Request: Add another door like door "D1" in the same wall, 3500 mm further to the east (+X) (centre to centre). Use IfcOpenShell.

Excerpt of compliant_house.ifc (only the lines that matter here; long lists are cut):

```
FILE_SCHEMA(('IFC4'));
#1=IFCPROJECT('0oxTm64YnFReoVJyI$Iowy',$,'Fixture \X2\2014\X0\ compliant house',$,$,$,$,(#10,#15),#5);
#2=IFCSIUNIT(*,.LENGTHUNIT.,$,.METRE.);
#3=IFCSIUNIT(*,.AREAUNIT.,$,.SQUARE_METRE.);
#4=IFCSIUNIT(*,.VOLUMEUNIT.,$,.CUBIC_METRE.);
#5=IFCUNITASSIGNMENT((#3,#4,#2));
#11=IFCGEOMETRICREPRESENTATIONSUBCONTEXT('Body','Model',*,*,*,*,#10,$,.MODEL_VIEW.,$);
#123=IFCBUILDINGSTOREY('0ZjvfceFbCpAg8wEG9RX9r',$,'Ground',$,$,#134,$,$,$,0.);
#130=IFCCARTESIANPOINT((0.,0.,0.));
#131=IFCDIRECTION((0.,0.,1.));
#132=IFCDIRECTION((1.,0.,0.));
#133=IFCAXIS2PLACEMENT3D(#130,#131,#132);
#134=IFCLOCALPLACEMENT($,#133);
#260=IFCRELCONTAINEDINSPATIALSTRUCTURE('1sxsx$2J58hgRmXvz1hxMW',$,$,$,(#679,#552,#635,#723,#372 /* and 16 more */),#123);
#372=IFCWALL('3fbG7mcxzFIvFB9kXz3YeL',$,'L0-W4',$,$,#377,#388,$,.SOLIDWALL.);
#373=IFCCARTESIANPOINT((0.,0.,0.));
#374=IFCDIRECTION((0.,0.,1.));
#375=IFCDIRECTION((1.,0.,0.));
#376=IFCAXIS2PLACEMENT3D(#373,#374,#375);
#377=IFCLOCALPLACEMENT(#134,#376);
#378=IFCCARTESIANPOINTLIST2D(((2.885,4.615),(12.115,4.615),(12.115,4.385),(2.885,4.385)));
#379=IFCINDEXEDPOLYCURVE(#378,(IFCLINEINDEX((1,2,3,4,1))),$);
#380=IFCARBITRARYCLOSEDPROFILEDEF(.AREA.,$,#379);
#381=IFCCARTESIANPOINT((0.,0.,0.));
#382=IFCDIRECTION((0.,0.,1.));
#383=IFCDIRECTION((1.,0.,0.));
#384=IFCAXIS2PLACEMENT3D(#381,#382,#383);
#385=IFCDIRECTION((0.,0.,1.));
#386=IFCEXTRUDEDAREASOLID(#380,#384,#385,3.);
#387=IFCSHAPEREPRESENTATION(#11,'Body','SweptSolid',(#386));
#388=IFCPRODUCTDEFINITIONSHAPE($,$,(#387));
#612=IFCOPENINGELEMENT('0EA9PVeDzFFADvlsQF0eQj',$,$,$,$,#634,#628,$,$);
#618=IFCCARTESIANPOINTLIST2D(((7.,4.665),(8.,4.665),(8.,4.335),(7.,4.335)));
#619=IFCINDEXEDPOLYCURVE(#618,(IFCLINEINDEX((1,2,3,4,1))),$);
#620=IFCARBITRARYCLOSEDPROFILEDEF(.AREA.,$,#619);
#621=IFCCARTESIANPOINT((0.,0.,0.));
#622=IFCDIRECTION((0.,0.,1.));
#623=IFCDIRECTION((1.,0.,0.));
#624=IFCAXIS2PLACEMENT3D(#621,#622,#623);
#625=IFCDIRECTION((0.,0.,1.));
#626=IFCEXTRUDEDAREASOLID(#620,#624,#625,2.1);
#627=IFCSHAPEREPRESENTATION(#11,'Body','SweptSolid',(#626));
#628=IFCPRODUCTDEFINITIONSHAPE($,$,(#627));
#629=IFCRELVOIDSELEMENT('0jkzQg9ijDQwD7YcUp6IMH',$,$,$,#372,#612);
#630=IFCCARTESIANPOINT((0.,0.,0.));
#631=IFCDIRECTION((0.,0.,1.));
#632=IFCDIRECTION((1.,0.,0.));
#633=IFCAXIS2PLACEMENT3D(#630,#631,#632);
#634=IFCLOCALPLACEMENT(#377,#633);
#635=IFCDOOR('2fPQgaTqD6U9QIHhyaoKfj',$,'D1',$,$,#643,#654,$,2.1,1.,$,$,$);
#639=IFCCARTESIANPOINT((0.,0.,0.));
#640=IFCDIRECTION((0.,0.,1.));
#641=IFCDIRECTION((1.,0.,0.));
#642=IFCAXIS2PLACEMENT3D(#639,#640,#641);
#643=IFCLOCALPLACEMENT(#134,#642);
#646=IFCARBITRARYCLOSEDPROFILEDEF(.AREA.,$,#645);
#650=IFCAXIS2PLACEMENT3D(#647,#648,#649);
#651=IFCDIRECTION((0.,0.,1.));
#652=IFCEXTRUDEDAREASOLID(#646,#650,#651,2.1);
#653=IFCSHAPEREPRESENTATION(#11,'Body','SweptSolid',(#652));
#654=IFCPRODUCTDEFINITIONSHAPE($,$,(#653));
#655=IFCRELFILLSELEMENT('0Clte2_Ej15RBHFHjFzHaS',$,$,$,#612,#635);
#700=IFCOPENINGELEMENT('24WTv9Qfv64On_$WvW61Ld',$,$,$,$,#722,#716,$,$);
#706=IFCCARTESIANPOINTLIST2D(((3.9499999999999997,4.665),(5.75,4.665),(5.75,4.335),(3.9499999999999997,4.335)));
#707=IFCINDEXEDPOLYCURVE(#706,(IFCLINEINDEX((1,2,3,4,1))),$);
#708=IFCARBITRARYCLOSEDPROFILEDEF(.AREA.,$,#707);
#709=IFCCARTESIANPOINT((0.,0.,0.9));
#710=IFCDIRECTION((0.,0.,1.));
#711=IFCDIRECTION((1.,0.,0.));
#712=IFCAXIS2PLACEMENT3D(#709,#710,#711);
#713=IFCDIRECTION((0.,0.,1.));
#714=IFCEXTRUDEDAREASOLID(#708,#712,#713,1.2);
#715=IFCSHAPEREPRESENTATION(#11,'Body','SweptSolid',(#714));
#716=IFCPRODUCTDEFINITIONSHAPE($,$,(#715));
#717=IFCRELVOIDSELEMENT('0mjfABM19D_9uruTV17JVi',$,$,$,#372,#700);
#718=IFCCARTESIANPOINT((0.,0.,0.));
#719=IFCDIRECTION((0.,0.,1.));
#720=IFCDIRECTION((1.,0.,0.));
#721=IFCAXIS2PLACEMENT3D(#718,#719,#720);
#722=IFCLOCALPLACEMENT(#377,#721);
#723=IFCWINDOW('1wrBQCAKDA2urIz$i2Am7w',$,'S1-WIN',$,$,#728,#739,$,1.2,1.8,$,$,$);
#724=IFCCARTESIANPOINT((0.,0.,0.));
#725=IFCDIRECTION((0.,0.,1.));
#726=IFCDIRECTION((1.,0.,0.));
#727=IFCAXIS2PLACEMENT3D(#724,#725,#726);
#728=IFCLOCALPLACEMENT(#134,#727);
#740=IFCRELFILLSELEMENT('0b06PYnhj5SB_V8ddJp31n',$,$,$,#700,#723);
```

```python
import ifcopenshell
import ifcopenshell.api.feature
import ifcopenshell.api.geometry
import ifcopenshell.api.root
import ifcopenshell.geom
import ifcopenshell.util.element
import ifcopenshell.util.placement
import ifcopenshell.util.shape
import ifcopenshell.util.unit

model = ifcopenshell.open("compliant_house.ifc")
unit_scale = ifcopenshell.util.unit.calculate_unit_scale(model)
settings = ifcopenshell.geom.settings()


def volume(element):
    """Net volume in cubic metres, openings subtracted."""
    shape = ifcopenshell.geom.create_shape(settings, element)
    return ifcopenshell.util.shape.get_volume(shape.geometry)


door = model.by_guid("2fPQgaTqD6U9QIHhyaoKfj")
opening = door.FillsVoids[0].RelatingOpeningElement
wall = opening.VoidsElements[0].RelatingBuildingElement
before = volume(wall)
shift = ifcopenshell.util.placement.get_local_placement(wall.ObjectPlacement)[:3, 0] * 3.5 / unit_scale

# copy_class copies the void relationship, type, container and properties, but no geometry.
new_opening = ifcopenshell.api.root.copy_class(model, product=opening)
new_opening.Representation = ifcopenshell.util.element.copy_deep(
    model, opening.Representation, exclude=["IfcGeometricRepresentationContext", "IfcRepresentationMap"]
)
new_door = ifcopenshell.api.root.copy_class(model, product=door)
new_door.Representation = ifcopenshell.util.element.copy_deep(
    model, door.Representation, exclude=["IfcGeometricRepresentationContext", "IfcRepresentationMap"]
)
ifcopenshell.api.feature.add_filling(model, opening=new_opening, element=new_door)

for old, new in ((opening, new_opening), (door, new_door)):
    matrix = ifcopenshell.util.placement.get_local_placement(old.ObjectPlacement)
    matrix[:3, 3] += shift
    ifcopenshell.api.geometry.edit_object_placement(model, product=new, matrix=matrix, is_si=False)

after = volume(wall)

print(f"wall volume {before:.3f} -> {after:.3f} m3")

model.write("compliant_house_rev.ifc")
```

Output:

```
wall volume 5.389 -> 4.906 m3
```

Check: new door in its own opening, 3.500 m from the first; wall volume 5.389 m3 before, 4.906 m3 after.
